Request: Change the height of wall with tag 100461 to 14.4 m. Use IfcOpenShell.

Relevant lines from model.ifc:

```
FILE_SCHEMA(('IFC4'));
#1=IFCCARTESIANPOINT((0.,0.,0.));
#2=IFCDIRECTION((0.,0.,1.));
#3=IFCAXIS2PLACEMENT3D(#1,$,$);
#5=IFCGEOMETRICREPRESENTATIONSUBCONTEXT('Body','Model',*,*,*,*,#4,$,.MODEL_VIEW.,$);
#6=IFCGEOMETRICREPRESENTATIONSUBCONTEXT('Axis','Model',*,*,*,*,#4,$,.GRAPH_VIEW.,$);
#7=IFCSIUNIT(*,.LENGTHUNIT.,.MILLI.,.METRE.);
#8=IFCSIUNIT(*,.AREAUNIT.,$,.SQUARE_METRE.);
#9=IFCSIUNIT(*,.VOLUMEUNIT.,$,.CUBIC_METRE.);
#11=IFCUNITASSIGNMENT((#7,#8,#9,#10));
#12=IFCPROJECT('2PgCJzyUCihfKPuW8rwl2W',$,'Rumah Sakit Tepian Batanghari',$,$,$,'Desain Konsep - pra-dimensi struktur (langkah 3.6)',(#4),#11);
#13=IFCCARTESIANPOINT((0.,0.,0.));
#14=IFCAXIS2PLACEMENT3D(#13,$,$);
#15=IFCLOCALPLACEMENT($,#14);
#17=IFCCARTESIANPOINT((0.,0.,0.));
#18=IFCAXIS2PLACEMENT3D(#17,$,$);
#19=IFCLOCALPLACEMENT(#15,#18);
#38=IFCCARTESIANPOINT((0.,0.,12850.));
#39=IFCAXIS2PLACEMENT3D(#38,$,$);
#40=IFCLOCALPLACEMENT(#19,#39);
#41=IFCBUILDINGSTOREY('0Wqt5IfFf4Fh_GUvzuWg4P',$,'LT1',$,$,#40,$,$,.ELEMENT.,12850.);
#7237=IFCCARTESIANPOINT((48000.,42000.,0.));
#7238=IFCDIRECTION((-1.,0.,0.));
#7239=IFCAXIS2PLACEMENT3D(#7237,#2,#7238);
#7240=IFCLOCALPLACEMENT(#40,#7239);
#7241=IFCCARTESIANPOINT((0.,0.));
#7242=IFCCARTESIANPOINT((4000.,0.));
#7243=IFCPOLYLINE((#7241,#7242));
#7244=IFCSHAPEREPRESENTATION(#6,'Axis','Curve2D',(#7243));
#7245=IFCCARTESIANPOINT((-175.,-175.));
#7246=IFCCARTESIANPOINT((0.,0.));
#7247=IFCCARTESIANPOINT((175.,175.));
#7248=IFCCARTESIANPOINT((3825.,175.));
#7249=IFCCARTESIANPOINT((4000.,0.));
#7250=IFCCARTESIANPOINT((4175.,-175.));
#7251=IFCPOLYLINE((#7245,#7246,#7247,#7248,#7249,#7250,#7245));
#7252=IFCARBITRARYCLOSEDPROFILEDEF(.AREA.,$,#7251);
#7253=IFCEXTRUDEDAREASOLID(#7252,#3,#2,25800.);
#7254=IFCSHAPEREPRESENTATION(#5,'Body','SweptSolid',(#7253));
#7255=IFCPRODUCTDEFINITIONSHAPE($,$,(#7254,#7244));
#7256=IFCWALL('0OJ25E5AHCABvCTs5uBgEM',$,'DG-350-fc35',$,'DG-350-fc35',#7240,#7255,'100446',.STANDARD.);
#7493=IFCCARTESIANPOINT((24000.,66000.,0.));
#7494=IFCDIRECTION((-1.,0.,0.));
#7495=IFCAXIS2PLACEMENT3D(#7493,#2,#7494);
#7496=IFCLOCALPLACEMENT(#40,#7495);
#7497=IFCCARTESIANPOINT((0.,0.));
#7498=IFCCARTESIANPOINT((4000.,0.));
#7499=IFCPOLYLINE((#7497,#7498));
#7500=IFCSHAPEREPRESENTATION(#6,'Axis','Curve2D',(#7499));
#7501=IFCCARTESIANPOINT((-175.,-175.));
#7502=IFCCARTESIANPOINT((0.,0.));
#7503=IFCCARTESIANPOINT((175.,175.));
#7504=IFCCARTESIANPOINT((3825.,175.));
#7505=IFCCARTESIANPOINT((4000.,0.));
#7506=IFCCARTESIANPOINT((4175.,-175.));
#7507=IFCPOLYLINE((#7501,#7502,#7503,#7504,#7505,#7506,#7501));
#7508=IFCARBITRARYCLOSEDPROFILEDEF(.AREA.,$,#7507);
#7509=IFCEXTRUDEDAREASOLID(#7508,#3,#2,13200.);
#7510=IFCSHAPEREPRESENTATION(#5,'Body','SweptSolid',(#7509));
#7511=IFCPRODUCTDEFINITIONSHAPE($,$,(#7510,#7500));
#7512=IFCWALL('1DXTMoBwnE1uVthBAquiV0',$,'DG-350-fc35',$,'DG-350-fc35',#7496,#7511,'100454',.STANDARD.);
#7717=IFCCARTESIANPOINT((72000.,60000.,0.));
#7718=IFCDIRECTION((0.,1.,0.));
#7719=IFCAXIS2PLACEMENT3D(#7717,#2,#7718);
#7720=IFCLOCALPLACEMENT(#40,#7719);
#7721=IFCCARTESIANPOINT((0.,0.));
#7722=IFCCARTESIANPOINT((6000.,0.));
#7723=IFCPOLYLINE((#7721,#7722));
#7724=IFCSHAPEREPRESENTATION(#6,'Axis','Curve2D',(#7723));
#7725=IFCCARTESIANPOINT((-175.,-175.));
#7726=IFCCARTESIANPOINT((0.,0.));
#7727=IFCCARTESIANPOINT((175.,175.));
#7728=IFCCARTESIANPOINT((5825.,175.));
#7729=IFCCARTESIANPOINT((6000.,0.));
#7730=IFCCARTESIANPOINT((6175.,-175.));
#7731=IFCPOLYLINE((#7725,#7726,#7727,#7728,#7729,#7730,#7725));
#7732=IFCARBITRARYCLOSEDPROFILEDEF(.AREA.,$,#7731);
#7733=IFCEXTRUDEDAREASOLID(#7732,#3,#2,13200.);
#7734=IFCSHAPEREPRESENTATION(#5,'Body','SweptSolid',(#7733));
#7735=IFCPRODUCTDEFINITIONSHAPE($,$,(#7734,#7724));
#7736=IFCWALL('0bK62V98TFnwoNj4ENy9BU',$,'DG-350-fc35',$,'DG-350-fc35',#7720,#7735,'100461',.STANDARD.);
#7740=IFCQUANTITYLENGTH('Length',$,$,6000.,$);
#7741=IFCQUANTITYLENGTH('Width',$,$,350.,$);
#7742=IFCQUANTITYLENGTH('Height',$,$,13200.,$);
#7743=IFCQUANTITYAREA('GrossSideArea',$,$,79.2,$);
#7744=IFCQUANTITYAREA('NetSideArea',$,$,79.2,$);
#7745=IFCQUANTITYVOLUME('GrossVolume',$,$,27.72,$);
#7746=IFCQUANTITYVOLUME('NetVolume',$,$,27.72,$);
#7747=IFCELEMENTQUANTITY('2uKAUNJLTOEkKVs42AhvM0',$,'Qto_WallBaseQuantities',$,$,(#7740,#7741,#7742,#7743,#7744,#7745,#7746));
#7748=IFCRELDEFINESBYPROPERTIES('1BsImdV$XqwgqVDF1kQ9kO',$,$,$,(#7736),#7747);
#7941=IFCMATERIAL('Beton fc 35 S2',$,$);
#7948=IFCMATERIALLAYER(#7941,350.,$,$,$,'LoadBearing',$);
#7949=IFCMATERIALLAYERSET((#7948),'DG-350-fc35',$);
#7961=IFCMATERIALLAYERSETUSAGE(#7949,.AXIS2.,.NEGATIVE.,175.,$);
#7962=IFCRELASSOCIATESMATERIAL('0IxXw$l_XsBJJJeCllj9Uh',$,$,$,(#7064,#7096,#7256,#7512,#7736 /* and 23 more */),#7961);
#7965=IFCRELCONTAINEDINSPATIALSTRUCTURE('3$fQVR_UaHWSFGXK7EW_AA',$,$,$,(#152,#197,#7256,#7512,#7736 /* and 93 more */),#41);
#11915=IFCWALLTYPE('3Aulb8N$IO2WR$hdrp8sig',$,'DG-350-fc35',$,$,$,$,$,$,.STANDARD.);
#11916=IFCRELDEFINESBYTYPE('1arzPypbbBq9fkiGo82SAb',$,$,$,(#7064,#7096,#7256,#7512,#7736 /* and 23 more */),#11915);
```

```python
import ifcopenshell
import ifcopenshell.api.pset
import ifcopenshell.geom
import ifcopenshell.util.element
import ifcopenshell.util.representation
import ifcopenshell.util.shape
import ifcopenshell.util.unit

model = ifcopenshell.open("model.ifc")
unit_scale = ifcopenshell.util.unit.calculate_unit_scale(model)
area_scale = ifcopenshell.util.unit.calculate_unit_scale(model, "AREAUNIT")
volume_scale = ifcopenshell.util.unit.calculate_unit_scale(model, "VOLUMEUNIT")
settings = ifcopenshell.geom.settings()


def volume(element):
    """Net volume in cubic metres, openings subtracted."""
    shape = ifcopenshell.geom.create_shape(settings, element)
    return ifcopenshell.util.shape.get_volume(shape.geometry)


wall = model.by_guid("0bK62V98TFnwoNj4ENy9BU")
before = volume(wall)

body = ifcopenshell.util.representation.get_representation(wall, "Model", "Body")
solid = body.Items[0]
old_height = solid.Depth
solid.Depth = 14.4 / unit_scale
after = volume(wall)
thickness = 0.35  # wall thickness in metres

# Update the stored height, areas and volumes.
qto = model.by_id(ifcopenshell.util.element.get_pset(wall, "Qto_WallBaseQuantities", should_inherit=False)["id"])
ifcopenshell.api.pset.edit_qto(model, qto=qto, properties={
    "Height": solid.Depth,
    "GrossSideArea": ifcopenshell.util.element.get_pset(wall, "Qto_WallBaseQuantities", "GrossSideArea") * solid.Depth / old_height,
    "NetSideArea": after / thickness / area_scale,
    "GrossVolume": ifcopenshell.util.element.get_pset(wall, "Qto_WallBaseQuantities", "GrossVolume") * solid.Depth / old_height,
    "NetVolume": after / volume_scale,
})

print(f"height {old_height:g} -> {solid.Depth:g}, volume {before:.3f} -> {after:.3f} m3")

model.write("model-out.ifc")
```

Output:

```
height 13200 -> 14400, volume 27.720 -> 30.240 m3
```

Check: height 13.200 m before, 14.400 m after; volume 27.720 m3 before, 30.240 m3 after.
